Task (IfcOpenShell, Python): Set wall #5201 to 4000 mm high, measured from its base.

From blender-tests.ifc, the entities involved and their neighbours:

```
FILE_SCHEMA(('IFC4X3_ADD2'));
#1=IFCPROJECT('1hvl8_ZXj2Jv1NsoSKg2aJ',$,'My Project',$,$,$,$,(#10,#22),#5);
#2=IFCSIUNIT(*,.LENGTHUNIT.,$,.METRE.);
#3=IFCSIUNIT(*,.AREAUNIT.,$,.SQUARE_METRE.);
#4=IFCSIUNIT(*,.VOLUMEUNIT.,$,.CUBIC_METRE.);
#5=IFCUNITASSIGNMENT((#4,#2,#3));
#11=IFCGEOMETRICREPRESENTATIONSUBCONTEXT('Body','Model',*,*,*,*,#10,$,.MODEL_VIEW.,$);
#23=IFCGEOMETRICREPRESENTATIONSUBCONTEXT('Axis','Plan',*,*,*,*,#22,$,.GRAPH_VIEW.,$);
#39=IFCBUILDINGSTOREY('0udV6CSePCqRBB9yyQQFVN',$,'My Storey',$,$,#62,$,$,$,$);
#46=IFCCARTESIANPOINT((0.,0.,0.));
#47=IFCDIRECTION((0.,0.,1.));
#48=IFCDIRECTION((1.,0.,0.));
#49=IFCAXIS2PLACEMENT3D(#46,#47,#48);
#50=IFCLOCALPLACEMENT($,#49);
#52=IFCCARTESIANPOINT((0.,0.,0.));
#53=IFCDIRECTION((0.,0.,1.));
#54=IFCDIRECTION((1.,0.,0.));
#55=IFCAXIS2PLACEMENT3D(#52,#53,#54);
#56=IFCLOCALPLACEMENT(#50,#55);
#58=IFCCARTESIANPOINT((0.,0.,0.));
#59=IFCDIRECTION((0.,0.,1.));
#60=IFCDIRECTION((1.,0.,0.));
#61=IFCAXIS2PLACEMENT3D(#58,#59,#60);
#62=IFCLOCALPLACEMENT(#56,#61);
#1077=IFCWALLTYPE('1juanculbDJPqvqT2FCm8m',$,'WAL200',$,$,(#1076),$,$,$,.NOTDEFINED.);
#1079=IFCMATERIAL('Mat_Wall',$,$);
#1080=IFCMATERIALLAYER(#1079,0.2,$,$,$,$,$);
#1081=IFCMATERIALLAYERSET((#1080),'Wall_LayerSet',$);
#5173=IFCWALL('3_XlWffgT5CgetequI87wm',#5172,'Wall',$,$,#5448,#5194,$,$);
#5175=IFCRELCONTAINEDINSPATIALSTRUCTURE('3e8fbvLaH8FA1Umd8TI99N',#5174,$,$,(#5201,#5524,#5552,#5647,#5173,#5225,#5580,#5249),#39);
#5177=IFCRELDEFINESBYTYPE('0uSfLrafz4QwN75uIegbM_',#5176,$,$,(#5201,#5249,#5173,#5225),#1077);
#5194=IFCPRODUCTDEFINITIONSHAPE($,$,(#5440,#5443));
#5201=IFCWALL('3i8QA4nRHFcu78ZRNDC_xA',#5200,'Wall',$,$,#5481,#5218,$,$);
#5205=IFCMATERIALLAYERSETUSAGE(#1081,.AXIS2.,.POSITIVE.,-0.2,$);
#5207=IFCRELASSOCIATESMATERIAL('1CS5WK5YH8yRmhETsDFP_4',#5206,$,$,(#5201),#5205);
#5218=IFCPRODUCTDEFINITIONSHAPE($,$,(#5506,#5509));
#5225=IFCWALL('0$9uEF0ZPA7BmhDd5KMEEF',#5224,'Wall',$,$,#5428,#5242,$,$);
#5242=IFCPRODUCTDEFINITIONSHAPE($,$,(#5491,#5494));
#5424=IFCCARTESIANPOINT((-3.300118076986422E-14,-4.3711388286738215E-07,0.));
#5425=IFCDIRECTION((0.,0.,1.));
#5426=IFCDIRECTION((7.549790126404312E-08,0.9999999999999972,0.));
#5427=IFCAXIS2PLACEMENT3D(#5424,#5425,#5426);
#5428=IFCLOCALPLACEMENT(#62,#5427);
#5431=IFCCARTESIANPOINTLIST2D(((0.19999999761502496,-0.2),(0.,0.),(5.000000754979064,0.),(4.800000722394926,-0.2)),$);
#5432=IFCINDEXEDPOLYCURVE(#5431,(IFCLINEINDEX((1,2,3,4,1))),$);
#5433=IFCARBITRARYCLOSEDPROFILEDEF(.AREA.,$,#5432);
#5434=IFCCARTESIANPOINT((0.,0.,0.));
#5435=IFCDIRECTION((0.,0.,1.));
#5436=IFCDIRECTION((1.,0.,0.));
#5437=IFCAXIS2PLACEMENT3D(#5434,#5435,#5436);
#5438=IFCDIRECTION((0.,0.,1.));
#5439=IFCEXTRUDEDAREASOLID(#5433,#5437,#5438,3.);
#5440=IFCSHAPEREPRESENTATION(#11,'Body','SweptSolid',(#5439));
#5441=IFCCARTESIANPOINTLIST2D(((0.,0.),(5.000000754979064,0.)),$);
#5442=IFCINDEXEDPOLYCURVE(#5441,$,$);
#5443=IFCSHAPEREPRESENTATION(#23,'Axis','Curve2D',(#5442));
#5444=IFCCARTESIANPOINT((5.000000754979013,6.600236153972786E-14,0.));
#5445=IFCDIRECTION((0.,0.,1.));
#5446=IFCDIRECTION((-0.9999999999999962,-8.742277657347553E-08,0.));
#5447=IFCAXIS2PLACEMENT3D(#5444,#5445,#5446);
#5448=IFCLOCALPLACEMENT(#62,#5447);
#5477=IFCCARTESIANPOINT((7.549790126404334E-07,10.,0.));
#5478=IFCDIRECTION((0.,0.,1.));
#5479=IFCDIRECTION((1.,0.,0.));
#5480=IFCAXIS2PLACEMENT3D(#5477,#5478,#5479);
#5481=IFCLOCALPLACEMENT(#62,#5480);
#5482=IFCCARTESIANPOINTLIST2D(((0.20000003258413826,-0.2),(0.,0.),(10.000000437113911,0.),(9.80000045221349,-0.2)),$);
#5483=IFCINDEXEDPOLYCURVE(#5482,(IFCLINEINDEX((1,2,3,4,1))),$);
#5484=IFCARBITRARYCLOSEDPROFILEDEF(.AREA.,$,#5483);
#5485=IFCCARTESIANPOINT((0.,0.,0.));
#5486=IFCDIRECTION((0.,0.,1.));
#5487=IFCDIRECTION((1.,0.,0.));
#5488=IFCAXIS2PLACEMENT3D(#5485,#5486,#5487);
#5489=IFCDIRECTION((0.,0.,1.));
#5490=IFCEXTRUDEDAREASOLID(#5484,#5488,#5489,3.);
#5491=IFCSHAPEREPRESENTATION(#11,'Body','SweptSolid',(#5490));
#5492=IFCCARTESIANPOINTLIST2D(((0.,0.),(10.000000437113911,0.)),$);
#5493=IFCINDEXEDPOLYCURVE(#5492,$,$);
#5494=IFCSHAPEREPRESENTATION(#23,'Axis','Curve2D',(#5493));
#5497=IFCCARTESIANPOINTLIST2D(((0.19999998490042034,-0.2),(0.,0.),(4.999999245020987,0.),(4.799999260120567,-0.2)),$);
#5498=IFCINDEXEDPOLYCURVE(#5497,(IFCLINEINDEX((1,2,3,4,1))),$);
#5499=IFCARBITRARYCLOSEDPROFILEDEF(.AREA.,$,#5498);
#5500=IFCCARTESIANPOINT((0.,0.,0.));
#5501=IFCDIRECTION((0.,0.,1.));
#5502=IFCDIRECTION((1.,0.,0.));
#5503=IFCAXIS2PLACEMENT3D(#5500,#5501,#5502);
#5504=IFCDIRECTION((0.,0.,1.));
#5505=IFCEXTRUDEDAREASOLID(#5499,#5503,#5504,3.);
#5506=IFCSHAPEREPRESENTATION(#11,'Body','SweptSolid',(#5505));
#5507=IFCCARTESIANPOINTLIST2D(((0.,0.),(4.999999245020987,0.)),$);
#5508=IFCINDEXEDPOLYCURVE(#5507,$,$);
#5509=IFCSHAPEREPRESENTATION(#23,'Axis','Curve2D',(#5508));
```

```python
import ifcopenshell
import ifcopenshell.geom
import ifcopenshell.util.representation
import ifcopenshell.util.shape
import ifcopenshell.util.unit

model = ifcopenshell.open("blender-tests.ifc")
unit_scale = ifcopenshell.util.unit.calculate_unit_scale(model)
settings = ifcopenshell.geom.settings()


def volume(element):
    """Net volume in cubic metres, openings subtracted."""
    shape = ifcopenshell.geom.create_shape(settings, element)
    return ifcopenshell.util.shape.get_volume(shape.geometry)


wall = model.by_guid("3i8QA4nRHFcu78ZRNDC_xA")
before = volume(wall)

body = ifcopenshell.util.representation.get_representation(wall, "Model", "Body")
solid = body.Items[0]
old_height = solid.Depth
solid.Depth = 4 / unit_scale
after = volume(wall)

print(f"height {old_height:g} -> {solid.Depth:g}, volume {before:.3f} -> {after:.3f} m3")

model.write("blender-tests_rev.ifc")
```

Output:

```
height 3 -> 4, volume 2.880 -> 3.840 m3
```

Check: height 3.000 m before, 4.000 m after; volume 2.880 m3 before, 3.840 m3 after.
